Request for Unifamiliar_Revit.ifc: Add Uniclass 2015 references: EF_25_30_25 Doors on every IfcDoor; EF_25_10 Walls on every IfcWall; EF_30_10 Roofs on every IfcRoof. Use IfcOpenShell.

First a look at what the model holds.

```python
import ifcopenshell

model = ifcopenshell.open("Unifamiliar_Revit.ifc")
print(model.schema)
print("classifications:", [c.Name for c in model.by_type("IfcClassification")])
for ifc_class in ("IfcDoor", "IfcRoof", "IfcStair", "IfcWall", "IfcWindow"):
    print(ifc_class, len(model.by_type(ifc_class)))
```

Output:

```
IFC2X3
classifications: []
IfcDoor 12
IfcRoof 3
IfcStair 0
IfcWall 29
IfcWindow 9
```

```python
import ifcopenshell
import ifcopenshell.api.classification

model = ifcopenshell.open("Unifamiliar_Revit.ifc")

# IFC2X3 requires Source and Edition and has no link from the project to the system.
system = model.create_entity("IfcClassification", Source="NBS", Edition="2015", Name="Uniclass 2015")

codes = {
    "IfcDoor": ("EF_25_30_25", "Doors"),
    "IfcWall": ("EF_25_10", "Walls"),
    "IfcRoof": ("EF_30_10", "Roofs"),
}
for ifc_class, (code, name) in codes.items():
    products = model.by_type(ifc_class)
    ifcopenshell.api.classification.add_reference(
        model, products=products, classification=system, identification=code, name=name
    )
    print(code, len(products))

model.write("Unifamiliar_Revit_updated.ifc")
```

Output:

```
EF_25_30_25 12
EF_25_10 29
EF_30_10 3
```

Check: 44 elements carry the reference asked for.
